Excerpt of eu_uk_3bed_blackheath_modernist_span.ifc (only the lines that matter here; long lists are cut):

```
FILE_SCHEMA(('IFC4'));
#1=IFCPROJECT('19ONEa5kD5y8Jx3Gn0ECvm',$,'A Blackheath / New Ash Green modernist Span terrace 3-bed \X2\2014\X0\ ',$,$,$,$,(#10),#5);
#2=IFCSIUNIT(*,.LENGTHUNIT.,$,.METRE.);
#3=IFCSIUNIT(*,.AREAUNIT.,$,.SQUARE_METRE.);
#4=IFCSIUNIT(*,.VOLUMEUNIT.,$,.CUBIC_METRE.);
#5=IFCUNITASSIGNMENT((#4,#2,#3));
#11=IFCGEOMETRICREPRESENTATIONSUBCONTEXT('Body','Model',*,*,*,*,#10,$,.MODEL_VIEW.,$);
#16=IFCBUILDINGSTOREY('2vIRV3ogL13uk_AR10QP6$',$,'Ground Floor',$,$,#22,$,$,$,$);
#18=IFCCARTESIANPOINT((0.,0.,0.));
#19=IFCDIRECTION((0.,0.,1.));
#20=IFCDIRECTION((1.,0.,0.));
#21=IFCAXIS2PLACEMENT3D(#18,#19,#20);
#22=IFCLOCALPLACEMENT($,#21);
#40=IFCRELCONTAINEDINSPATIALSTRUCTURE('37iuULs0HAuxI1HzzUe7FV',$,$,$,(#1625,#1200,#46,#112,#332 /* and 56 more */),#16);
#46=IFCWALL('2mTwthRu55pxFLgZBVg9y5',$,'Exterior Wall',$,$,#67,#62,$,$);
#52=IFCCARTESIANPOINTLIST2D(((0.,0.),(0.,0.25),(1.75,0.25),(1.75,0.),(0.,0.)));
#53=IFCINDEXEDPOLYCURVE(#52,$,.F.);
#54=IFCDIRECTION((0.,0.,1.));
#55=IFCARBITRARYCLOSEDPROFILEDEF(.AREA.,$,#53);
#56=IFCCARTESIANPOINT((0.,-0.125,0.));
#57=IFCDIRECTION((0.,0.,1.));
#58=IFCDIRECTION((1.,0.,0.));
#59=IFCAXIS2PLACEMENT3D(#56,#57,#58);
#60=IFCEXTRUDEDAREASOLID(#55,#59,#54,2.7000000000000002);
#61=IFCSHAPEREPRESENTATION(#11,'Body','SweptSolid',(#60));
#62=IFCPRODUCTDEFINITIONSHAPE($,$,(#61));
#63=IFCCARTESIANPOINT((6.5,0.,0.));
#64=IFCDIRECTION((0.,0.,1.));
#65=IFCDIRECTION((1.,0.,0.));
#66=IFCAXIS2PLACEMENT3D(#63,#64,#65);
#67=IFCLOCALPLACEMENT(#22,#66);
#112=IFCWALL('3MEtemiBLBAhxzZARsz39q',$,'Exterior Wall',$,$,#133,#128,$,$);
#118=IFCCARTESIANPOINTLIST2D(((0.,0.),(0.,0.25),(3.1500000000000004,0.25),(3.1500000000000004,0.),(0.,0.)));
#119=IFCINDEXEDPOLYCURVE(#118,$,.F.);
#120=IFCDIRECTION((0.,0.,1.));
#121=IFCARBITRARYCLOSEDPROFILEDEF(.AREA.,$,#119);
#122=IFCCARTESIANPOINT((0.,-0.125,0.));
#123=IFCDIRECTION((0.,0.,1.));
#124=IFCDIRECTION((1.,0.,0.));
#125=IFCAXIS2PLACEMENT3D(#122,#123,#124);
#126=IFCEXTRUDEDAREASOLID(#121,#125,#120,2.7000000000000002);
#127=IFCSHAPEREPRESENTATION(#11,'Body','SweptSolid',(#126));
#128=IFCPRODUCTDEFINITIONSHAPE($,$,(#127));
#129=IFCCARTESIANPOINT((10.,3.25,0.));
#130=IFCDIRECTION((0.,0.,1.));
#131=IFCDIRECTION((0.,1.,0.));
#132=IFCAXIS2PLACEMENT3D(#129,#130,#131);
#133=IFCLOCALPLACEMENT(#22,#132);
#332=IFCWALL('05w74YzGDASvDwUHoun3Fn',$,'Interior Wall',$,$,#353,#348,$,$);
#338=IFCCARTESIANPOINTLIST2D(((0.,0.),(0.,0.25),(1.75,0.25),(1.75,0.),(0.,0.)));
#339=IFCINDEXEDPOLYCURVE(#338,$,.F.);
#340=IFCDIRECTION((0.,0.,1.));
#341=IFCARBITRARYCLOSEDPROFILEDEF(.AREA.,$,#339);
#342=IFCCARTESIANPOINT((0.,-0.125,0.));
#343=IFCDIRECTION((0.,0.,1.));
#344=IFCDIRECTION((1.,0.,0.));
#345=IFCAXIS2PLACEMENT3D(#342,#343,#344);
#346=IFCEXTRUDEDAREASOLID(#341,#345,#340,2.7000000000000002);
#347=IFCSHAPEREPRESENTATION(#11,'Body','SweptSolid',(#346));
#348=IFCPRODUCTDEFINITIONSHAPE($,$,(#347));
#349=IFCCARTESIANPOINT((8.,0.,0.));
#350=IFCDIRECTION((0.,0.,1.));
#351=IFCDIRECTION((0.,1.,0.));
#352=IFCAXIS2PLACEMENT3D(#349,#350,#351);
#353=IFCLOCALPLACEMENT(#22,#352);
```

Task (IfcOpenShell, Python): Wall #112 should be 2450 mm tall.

```python
import ifcopenshell
import ifcopenshell.geom
import ifcopenshell.util.representation
import ifcopenshell.util.shape

model = ifcopenshell.open("eu_uk_3bed_blackheath_modernist_span.ifc")
settings = ifcopenshell.geom.settings()


def volume(element):
    """Net volume in cubic metres, openings subtracted."""
    shape = ifcopenshell.geom.create_shape(settings, element)
    return ifcopenshell.util.shape.get_volume(shape.geometry)


wall = model.by_guid("3MEtemiBLBAhxzZARsz39q")
before = volume(wall)

body = ifcopenshell.util.representation.get_representation(wall, "Model", "Body")
solid = body.Items[0]
old_height = solid.Depth
solid.Depth = 2.45
after = volume(wall)

print(f"height {old_height:g} -> {solid.Depth:g}, volume {before:.3f} -> {after:.3f} m3")

model.write("eu_uk_3bed_blackheath_modernist_span-out.ifc")
```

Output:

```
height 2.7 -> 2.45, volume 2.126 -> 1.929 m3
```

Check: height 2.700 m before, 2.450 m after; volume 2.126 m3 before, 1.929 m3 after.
